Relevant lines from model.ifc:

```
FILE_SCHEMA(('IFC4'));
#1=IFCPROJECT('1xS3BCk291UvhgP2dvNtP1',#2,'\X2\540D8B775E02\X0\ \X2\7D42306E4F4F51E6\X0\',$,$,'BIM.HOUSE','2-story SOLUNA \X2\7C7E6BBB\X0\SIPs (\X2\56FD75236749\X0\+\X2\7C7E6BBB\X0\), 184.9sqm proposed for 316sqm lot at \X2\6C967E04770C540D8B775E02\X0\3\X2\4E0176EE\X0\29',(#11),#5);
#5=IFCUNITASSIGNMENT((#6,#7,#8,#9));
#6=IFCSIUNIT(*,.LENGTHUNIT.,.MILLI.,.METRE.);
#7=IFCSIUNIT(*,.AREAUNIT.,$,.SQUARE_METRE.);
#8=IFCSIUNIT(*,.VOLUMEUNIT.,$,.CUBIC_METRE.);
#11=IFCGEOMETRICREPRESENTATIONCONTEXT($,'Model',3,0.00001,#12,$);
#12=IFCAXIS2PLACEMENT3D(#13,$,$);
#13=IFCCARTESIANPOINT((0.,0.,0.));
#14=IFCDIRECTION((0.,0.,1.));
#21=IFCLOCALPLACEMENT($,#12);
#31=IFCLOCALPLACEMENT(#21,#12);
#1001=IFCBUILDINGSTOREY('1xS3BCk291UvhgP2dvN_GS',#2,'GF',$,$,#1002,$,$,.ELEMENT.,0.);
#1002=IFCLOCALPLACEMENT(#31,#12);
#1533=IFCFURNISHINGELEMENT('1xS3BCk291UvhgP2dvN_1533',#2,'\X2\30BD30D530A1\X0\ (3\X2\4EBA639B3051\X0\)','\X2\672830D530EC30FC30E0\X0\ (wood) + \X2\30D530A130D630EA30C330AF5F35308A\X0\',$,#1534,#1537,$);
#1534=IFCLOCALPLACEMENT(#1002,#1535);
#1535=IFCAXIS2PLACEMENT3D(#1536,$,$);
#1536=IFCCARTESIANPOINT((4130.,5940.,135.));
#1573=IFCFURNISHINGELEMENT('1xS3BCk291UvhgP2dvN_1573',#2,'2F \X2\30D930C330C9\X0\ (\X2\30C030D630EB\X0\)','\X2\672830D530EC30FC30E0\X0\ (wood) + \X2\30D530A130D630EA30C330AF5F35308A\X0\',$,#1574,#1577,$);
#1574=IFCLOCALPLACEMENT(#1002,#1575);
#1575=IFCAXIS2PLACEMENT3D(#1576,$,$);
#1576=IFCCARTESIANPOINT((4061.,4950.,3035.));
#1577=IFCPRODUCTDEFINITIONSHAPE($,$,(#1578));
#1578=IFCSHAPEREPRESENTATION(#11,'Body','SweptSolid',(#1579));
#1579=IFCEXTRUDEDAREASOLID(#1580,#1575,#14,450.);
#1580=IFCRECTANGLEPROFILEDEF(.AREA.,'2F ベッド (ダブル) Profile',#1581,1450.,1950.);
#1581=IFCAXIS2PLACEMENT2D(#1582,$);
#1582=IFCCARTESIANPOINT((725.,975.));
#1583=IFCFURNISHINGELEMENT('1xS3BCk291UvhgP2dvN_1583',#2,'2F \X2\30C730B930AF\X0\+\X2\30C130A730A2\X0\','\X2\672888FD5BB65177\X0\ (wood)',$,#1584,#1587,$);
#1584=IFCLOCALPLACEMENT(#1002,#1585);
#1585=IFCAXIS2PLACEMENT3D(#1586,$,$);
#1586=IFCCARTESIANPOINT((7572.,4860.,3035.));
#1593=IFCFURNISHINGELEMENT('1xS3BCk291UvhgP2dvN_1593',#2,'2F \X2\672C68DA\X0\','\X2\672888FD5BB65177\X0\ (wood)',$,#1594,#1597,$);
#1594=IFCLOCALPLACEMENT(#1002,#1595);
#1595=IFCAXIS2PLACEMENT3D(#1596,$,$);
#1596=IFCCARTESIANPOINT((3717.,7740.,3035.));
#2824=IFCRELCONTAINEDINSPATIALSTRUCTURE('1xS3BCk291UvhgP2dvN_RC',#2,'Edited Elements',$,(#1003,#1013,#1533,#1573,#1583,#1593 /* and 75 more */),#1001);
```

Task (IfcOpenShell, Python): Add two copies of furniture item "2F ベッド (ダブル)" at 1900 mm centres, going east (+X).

```python
import numpy as np
import ifcopenshell
import ifcopenshell.api.geometry
import ifcopenshell.api.root
import ifcopenshell.util.element
import ifcopenshell.util.placement
import ifcopenshell.util.unit

model = ifcopenshell.open("model.ifc")
unit_scale = ifcopenshell.util.unit.calculate_unit_scale(model)


def reuse_history(source, copy):
    """copy_class also copies each property set's owner history, people and application; keep the originals."""
    for rel in copy.IsDefinedBy:
        if rel.is_a("IfcRelDefinesByProperties") and (history := rel.RelatingPropertyDefinition.OwnerHistory):
            rel.RelatingPropertyDefinition.OwnerHistory = source.OwnerHistory
            ifcopenshell.util.element.remove_deep2(model, history)


source = model.by_id(1573)
base = ifcopenshell.util.placement.get_local_placement(source.ObjectPlacement)
step = np.array([1.0, 0.0, 0.0]) * 1.9 / unit_scale

for i in range(1, 3):
    copy = ifcopenshell.api.root.copy_class(model, product=source)
    copy.Representation = ifcopenshell.util.element.copy_deep(
        model, source.Representation, exclude=["IfcGeometricRepresentationContext", "IfcRepresentationMap"]
    )
    reuse_history(source, copy)
    matrix = base.copy()
    matrix[:3, 3] += i * step
    print("added at", matrix[:3, 3].round(3) + 0.0)
    ifcopenshell.api.geometry.edit_object_placement(model, product=copy, matrix=matrix, is_si=False)

model.write("model_updated.ifc")
```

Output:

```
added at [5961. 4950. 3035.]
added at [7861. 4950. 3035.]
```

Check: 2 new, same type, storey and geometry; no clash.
